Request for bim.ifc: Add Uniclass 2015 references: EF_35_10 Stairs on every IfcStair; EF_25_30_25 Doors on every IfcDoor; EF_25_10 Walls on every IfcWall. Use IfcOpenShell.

First a look at what the model holds.

```python
import ifcopenshell

model = ifcopenshell.open("bim.ifc")
print(model.schema)
print("classifications:", [c.Name for c in model.by_type("IfcClassification")])
for ifc_class in ("IfcDoor", "IfcRoof", "IfcStair", "IfcWall", "IfcWindow"):
    print(ifc_class, len(model.by_type(ifc_class)))
```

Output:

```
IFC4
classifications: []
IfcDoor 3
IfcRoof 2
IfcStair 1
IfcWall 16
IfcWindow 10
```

```python
import ifcopenshell
import ifcopenshell.api.classification

model = ifcopenshell.open("bim.ifc")

system = ifcopenshell.api.classification.add_classification(model, classification="Uniclass 2015")

codes = {
    "IfcStair": ("EF_35_10", "Stairs"),
    "IfcDoor": ("EF_25_30_25", "Doors"),
    "IfcWall": ("EF_25_10", "Walls"),
}
for ifc_class, (code, name) in codes.items():
    products = model.by_type(ifc_class)
    ifcopenshell.api.classification.add_reference(
        model, products=products, classification=system, identification=code, name=name
    )
    print(code, len(products))

model.write("bim-out.ifc")
```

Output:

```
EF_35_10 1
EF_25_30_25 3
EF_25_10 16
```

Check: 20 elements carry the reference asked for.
